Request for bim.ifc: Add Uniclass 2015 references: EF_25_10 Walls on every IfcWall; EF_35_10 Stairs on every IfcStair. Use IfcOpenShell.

First a look at what the model holds.

```python
import ifcopenshell

model = ifcopenshell.open("bim.ifc")
print(model.schema)
print("classifications:", [c.Name for c in model.by_type("IfcClassification")])
for ifc_class in ("IfcDoor", "IfcRoof", "IfcStair", "IfcWall", "IfcWindow"):
    print(ifc_class, len(model.by_type(ifc_class)))
```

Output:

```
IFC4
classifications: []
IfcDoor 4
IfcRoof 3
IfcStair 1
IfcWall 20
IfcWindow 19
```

```python
import ifcopenshell
import ifcopenshell.api.classification

model = ifcopenshell.open("bim.ifc")

system = ifcopenshell.api.classification.add_classification(model, classification="Uniclass 2015")

codes = {
    "IfcWall": ("EF_25_10", "Walls"),
    "IfcStair": ("EF_35_10", "Stairs"),
}
for ifc_class, (code, name) in codes.items():
    products = model.by_type(ifc_class)
    ifcopenshell.api.classification.add_reference(
        model, products=products, classification=system, identification=code, name=name
    )
    print(code, len(products))

model.write("bim_updated.ifc")
```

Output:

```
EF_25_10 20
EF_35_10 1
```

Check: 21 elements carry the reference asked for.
